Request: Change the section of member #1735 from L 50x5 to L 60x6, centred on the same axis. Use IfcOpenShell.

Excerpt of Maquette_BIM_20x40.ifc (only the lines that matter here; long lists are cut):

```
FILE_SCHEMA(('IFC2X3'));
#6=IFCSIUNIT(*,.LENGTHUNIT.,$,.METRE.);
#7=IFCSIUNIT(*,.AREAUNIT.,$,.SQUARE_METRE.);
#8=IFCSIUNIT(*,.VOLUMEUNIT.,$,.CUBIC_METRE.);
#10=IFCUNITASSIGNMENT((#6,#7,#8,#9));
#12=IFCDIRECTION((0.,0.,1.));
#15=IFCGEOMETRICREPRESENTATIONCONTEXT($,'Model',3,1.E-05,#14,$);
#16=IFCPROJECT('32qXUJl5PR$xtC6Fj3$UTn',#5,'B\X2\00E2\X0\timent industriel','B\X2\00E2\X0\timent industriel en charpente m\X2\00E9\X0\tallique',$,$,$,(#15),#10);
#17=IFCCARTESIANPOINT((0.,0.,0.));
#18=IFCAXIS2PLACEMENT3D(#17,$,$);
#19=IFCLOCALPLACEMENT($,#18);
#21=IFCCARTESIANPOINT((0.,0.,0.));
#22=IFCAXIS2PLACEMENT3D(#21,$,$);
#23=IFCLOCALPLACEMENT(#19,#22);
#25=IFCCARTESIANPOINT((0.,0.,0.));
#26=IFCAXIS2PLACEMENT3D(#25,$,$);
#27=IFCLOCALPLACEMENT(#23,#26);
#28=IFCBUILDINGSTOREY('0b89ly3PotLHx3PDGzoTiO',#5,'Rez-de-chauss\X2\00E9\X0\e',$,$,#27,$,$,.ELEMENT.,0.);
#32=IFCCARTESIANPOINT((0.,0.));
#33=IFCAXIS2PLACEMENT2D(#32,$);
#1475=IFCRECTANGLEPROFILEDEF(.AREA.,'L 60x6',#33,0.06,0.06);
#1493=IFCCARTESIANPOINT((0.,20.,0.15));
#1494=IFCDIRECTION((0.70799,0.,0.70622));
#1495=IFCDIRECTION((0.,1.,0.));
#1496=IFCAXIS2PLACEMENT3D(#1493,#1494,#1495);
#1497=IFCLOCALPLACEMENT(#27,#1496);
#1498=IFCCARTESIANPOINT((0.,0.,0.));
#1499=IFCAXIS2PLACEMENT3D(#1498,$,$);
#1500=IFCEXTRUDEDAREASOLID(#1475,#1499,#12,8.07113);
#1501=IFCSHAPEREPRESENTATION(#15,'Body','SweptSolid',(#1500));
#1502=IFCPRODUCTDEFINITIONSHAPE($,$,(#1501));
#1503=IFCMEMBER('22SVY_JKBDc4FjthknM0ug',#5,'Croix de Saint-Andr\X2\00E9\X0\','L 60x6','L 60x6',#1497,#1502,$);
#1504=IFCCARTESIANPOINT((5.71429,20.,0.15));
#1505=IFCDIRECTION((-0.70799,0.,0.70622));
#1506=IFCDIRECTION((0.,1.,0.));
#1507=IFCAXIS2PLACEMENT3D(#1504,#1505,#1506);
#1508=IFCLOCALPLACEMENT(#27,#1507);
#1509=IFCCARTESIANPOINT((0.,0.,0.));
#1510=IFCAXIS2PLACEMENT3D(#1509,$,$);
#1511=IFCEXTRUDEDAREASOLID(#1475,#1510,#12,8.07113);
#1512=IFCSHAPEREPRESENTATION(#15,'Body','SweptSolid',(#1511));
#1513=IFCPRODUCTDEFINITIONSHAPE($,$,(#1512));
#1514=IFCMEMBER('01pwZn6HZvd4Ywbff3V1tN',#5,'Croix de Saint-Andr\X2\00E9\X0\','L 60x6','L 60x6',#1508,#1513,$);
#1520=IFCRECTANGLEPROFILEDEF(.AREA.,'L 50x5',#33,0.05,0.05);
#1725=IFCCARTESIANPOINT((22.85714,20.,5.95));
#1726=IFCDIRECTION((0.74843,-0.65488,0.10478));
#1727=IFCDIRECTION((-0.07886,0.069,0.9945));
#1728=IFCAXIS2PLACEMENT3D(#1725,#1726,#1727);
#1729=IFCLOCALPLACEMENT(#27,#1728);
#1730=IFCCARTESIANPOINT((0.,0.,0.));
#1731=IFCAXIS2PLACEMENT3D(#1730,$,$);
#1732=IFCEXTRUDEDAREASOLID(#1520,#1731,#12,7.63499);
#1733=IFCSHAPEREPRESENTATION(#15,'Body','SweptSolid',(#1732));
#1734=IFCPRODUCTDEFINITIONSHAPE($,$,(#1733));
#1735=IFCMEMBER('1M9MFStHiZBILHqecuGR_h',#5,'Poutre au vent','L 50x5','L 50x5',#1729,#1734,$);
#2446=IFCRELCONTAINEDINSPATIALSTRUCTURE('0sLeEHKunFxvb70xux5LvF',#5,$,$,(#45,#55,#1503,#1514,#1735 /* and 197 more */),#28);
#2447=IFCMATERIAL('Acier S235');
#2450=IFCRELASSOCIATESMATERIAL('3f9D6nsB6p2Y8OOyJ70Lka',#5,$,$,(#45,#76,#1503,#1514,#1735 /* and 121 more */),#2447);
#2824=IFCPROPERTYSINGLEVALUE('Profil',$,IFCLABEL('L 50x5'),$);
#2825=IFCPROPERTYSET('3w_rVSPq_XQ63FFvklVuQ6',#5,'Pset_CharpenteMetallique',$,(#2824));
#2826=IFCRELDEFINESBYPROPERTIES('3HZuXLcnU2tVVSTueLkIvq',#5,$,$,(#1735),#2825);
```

```python
import ifcopenshell
import ifcopenshell.api.pset
import ifcopenshell.util.element

model = ifcopenshell.open("Maquette_BIM_20x40.ifc")

member = model.by_id(1735)
source = next(p for p in model.by_type("IfcRectangleProfileDef") if p.ProfileName == "L 60x6")

body = next(r for r in member.Representation.Representations if r.RepresentationIdentifier == "Body")
solid = body.Items[0]
old_profile = solid.SweptArea

# Copy the section's sizes but keep this member's own profile position.
profile = ifcopenshell.util.element.copy(model, source)
profile.Position = old_profile.Position
solid.SweptArea = profile
if not model.get_total_inverses(old_profile):
    ifcopenshell.util.element.remove_deep2(model, old_profile)
member.Description = member.Description.replace("L 50x5", "L 60x6")
member.ObjectType = member.ObjectType.replace("L 50x5", "L 60x6")
pset = model.by_id(ifcopenshell.util.element.get_pset(member, "Pset_CharpenteMetallique", should_inherit=False)["id"])
ifcopenshell.api.pset.edit_pset(model, pset=pset, properties={"Profil": "L 60x6"})

print(solid.SweptArea)

model.write("Maquette_BIM_20x40_updated.ifc")
```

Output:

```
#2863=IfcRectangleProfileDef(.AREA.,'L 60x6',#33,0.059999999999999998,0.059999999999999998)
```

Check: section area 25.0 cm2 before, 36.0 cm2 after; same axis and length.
